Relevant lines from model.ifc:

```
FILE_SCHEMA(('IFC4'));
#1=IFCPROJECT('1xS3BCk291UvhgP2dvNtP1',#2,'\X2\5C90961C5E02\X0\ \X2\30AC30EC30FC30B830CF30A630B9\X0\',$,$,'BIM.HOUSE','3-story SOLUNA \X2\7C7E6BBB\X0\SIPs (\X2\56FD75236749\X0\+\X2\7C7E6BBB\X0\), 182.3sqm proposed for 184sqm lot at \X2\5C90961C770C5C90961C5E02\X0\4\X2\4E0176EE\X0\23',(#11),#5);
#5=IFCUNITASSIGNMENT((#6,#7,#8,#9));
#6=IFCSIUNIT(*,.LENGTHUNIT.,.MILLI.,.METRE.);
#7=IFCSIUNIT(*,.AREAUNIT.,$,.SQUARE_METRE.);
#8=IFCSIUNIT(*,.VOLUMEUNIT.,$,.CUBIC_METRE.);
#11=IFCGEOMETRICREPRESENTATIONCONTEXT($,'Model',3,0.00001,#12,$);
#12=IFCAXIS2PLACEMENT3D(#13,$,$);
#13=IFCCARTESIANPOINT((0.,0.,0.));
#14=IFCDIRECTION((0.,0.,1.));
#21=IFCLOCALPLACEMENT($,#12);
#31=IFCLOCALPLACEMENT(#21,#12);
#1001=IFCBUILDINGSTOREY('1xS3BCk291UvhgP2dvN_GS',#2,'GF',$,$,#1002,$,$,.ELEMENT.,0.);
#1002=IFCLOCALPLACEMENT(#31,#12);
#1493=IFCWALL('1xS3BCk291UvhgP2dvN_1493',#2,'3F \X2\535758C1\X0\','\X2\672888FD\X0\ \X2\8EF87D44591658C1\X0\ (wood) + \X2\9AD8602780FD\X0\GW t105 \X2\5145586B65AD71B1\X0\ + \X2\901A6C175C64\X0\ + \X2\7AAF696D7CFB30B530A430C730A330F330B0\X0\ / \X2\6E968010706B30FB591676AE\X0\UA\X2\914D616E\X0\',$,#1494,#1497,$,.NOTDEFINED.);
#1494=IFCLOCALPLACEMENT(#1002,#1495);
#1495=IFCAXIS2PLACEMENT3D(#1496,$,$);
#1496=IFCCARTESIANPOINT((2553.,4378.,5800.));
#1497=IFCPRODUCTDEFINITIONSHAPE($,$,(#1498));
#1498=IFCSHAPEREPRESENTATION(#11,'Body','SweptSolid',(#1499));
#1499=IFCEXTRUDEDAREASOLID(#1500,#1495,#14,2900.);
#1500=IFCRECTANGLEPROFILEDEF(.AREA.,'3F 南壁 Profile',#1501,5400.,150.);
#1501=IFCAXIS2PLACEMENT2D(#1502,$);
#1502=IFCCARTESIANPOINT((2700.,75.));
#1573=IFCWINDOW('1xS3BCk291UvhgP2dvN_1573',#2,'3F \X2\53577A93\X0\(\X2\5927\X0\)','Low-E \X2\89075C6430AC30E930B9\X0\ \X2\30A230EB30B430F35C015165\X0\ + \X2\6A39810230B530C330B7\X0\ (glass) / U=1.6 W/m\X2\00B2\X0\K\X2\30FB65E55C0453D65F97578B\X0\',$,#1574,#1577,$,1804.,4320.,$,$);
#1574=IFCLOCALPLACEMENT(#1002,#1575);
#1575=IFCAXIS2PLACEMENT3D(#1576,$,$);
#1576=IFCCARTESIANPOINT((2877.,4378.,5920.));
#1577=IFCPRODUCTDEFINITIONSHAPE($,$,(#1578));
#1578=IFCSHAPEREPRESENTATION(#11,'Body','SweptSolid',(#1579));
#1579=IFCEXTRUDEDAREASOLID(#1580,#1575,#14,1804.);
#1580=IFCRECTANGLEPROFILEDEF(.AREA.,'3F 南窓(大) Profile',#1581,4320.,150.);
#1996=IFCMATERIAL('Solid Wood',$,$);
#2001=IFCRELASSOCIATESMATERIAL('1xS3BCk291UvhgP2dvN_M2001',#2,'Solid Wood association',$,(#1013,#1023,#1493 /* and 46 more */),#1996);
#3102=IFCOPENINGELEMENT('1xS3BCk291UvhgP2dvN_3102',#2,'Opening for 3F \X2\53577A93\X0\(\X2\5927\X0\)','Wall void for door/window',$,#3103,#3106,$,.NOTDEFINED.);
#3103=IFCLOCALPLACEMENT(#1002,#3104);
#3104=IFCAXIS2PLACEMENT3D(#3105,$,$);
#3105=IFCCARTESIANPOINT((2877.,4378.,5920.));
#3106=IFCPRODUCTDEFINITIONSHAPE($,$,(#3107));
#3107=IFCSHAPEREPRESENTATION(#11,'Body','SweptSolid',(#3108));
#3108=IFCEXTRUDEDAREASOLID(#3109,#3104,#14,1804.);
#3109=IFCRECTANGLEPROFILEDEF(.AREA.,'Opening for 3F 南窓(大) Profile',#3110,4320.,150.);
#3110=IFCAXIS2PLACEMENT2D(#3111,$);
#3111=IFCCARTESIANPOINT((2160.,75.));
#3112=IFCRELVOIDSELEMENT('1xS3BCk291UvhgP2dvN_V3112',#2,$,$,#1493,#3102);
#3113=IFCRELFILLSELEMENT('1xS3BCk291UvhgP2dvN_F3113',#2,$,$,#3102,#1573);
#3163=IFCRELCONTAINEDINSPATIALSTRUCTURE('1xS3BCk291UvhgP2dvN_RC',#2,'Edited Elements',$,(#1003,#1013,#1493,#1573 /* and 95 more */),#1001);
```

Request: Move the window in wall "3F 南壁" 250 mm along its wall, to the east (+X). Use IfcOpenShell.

```python
import ifcopenshell
import ifcopenshell.api.geometry
import ifcopenshell.util.placement

model = ifcopenshell.open("model.ifc")

window = model.by_guid("1xS3BCk291UvhgP2dvN_1573")
opening = window.FillsVoids[0].RelatingOpeningElement
wall = opening.VoidsElements[0].RelatingBuildingElement

wall_matrix = ifcopenshell.util.placement.get_local_placement(wall.ObjectPlacement)
shift = wall_matrix[:3, 0] * 250.0
before = ifcopenshell.util.placement.get_local_placement(window.ObjectPlacement)[:3, 3].copy()

# The window is not placed relative to its opening, so move both.
for product in (opening, window):
    matrix = ifcopenshell.util.placement.get_local_placement(product.ObjectPlacement)
    matrix[:3, 3] += shift
    ifcopenshell.api.geometry.edit_object_placement(model, product=product, matrix=matrix, is_si=False)

after = ifcopenshell.util.placement.get_local_placement(window.ObjectPlacement)[:3, 3]
print("window moved by", (after - before).round(3) + 0.0)

model.write("model_v2.ifc")
```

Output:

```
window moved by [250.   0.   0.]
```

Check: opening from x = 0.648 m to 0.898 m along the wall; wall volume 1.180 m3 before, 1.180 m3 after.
